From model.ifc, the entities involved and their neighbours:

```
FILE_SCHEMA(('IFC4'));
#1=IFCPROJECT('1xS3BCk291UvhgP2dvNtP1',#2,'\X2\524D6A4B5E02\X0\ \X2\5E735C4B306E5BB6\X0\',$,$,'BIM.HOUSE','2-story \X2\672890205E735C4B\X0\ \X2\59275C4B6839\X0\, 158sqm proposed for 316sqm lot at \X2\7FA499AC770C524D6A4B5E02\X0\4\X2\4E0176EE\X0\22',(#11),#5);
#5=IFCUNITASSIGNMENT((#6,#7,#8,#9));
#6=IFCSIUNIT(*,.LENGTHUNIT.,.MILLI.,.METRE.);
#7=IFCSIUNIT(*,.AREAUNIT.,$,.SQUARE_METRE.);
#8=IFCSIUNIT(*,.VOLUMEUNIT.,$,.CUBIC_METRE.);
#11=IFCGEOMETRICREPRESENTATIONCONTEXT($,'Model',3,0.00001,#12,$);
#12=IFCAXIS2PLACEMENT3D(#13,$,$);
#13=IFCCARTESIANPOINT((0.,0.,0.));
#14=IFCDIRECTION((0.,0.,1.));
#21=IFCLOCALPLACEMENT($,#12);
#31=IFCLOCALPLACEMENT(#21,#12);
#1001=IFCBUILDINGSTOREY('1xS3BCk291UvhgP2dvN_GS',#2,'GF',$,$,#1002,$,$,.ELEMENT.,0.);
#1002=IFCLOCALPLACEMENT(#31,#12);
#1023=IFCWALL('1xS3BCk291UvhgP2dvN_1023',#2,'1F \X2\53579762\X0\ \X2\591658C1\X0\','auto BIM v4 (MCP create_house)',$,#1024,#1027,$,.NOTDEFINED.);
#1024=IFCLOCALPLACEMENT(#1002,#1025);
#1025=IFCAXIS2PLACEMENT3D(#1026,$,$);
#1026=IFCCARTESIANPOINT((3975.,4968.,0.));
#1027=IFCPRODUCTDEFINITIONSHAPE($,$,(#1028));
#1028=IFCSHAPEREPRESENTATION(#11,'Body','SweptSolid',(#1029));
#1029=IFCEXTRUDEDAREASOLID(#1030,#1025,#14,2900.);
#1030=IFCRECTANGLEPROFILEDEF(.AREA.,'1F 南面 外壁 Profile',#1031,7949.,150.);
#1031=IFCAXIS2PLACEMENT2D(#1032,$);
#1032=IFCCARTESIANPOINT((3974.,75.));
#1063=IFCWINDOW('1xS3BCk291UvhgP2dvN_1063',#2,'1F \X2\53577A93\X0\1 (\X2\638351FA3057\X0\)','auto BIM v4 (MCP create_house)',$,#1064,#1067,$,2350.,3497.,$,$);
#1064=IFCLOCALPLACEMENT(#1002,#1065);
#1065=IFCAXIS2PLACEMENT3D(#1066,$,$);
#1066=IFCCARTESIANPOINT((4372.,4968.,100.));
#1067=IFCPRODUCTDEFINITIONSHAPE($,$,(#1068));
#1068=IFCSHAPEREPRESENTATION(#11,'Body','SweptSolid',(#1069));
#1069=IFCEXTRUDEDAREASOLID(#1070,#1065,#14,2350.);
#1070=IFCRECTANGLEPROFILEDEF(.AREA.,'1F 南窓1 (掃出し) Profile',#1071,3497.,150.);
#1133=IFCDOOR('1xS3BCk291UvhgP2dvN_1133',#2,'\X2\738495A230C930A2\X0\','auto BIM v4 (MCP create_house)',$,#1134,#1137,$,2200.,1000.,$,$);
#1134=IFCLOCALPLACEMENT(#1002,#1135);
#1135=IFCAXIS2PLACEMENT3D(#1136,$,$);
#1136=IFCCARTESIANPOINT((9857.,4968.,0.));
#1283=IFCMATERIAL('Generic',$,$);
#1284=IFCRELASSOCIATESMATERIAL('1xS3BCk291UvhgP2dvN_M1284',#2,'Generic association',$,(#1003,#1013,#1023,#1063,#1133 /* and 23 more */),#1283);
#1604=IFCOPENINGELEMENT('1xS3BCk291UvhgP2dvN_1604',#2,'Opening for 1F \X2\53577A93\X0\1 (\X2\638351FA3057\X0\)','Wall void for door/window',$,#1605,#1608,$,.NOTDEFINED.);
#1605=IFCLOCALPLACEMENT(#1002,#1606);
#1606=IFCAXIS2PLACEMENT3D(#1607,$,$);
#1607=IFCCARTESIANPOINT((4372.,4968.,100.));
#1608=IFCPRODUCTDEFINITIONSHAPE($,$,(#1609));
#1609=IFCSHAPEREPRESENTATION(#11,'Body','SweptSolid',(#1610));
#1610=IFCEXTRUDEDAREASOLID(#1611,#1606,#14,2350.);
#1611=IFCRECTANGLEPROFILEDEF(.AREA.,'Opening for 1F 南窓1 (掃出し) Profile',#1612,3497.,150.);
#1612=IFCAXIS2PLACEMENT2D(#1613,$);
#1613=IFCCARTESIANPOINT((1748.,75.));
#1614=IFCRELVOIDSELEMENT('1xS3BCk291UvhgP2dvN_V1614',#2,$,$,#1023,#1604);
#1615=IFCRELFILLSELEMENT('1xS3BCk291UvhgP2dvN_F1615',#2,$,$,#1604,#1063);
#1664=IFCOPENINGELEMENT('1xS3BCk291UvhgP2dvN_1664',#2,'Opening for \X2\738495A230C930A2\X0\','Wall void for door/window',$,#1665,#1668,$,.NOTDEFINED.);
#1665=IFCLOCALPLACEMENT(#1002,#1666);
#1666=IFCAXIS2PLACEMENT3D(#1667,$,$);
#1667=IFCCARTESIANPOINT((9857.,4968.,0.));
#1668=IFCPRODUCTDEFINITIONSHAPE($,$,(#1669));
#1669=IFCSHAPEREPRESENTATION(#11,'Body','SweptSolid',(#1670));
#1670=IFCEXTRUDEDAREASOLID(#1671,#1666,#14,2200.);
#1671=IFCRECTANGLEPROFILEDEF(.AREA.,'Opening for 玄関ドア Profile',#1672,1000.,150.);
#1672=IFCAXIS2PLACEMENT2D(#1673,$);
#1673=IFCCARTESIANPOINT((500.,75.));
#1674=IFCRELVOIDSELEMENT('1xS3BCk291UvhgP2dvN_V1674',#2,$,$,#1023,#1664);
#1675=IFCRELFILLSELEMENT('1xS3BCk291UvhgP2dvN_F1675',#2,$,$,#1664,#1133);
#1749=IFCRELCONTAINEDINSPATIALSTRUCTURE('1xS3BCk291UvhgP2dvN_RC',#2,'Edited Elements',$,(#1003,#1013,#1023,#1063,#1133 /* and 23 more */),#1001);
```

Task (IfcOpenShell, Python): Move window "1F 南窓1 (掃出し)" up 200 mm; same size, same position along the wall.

```python
import numpy as np
import ifcopenshell
import ifcopenshell.api.geometry
import ifcopenshell.util.placement
import ifcopenshell.util.unit

model = ifcopenshell.open("model.ifc")
unit_scale = ifcopenshell.util.unit.calculate_unit_scale(model)

window = model.by_guid("1xS3BCk291UvhgP2dvN_1063")
opening = window.FillsVoids[0].RelatingOpeningElement
dz = 0.2 / unit_scale

shift = np.array([0.0, 0.0, dz])
# The window is not placed relative to its opening, so move both.
for product in (opening, window):
    matrix = ifcopenshell.util.placement.get_local_placement(product.ObjectPlacement)
    matrix[:3, 3] += shift
    ifcopenshell.api.geometry.edit_object_placement(model, product=product, matrix=matrix, is_si=False)

print(f"moved by {dz * unit_scale:+.3f} m")

model.write("model_updated.ifc")
```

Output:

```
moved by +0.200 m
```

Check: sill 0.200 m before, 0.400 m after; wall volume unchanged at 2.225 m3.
